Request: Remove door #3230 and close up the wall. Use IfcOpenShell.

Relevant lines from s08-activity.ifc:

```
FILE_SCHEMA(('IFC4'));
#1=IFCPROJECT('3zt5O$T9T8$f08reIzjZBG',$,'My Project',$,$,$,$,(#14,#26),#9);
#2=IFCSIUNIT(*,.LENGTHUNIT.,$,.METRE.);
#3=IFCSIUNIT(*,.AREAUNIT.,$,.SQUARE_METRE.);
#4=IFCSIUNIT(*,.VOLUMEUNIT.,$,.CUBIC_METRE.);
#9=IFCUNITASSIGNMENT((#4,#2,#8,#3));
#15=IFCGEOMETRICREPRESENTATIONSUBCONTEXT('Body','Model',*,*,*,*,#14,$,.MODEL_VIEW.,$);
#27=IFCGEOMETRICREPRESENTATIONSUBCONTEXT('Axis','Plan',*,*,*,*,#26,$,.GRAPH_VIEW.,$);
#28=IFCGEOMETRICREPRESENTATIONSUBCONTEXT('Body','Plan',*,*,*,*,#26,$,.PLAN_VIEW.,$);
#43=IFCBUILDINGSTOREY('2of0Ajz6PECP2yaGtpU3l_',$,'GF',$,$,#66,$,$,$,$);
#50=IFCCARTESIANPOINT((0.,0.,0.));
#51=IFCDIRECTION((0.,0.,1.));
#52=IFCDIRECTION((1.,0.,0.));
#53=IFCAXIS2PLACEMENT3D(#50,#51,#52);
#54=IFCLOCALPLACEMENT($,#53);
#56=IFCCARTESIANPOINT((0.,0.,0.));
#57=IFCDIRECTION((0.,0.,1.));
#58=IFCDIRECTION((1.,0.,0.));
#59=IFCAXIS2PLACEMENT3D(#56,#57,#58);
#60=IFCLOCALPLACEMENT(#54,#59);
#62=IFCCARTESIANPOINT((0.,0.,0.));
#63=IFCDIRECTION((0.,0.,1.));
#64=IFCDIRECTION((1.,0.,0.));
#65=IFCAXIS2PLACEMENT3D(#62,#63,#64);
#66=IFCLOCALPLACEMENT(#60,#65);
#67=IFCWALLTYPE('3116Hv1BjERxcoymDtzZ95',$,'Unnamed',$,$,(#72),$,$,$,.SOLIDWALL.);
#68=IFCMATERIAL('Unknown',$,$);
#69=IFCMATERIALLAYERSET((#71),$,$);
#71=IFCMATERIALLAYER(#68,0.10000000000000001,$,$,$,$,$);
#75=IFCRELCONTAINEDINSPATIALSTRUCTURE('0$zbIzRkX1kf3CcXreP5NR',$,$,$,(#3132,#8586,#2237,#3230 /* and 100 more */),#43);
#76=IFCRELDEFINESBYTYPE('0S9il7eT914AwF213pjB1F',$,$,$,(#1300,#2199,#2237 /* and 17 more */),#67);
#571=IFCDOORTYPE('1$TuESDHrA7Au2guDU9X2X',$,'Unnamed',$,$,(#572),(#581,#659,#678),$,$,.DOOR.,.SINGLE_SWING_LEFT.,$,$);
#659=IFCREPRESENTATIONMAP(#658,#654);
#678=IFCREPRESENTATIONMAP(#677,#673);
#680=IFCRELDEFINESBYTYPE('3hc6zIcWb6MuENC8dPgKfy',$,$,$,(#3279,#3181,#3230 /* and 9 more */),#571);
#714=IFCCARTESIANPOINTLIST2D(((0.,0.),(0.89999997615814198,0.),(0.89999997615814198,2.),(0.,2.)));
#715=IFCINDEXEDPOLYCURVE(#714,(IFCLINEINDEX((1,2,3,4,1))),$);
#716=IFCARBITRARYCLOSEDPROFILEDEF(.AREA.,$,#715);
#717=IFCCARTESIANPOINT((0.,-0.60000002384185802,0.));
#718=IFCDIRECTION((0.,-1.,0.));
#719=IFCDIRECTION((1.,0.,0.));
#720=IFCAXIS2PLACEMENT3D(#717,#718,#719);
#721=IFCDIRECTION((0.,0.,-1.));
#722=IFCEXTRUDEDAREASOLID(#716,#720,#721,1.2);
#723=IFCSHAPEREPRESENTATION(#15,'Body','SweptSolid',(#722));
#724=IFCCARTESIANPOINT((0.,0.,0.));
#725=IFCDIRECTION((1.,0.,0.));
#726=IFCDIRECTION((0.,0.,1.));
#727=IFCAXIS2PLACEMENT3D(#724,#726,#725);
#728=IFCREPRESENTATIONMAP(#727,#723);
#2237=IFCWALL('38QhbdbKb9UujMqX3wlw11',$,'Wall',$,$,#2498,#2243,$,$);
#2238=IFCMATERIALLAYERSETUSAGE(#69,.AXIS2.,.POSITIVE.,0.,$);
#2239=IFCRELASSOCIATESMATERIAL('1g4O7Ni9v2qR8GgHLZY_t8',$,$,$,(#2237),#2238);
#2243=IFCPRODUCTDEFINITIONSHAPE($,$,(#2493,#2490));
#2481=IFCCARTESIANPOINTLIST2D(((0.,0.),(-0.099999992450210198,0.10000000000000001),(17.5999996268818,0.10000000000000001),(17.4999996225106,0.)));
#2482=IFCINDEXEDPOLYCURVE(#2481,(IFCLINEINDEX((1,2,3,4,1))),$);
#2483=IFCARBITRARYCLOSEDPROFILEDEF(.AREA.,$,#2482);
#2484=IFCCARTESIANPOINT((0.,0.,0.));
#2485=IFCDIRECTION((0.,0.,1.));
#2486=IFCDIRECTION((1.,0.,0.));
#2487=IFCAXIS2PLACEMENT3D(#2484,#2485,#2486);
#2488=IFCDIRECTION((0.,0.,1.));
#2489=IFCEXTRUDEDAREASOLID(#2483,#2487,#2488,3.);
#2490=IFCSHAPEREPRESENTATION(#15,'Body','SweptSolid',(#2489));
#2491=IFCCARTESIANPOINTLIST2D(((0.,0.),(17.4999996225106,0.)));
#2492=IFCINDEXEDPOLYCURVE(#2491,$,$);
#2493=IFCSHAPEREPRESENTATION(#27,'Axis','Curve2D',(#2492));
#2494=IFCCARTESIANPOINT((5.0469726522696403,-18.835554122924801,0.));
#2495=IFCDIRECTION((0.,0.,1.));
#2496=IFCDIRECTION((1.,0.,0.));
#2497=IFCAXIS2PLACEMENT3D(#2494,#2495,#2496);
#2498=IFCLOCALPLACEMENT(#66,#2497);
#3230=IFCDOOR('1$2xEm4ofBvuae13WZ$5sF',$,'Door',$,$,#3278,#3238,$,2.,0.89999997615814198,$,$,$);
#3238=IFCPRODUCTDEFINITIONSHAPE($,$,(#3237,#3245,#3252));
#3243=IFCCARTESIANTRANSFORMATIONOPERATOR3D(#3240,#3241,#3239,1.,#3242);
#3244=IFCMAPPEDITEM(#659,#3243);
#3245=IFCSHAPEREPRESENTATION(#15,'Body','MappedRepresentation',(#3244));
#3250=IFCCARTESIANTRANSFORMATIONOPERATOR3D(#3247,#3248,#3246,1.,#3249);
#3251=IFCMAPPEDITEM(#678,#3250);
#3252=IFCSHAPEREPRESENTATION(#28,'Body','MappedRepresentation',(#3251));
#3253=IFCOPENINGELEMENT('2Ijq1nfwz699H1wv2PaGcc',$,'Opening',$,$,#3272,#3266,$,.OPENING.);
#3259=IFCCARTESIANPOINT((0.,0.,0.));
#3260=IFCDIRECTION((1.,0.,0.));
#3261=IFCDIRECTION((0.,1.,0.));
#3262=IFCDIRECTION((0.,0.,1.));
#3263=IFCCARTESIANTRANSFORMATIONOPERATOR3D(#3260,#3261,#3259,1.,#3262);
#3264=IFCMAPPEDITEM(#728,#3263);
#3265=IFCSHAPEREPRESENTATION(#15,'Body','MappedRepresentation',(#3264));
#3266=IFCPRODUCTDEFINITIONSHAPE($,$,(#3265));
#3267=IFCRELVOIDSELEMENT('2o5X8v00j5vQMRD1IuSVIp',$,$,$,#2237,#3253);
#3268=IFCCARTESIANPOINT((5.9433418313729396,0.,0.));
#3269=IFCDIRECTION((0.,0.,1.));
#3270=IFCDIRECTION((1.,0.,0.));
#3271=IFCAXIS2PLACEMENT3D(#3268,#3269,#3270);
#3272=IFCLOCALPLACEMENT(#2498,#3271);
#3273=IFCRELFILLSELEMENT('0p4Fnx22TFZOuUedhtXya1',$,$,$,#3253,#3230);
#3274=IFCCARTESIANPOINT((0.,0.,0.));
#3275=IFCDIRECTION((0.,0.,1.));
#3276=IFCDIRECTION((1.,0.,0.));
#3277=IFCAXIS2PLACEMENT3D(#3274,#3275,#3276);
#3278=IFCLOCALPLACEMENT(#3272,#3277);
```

```python
import ifcopenshell
import ifcopenshell.api.feature
import ifcopenshell.api.root
import ifcopenshell.geom
import ifcopenshell.util.shape

model = ifcopenshell.open("s08-activity.ifc")
settings = ifcopenshell.geom.settings()


def volume(element):
    """Net volume in cubic metres, openings subtracted."""
    shape = ifcopenshell.geom.create_shape(settings, element)
    return ifcopenshell.util.shape.get_volume(shape.geometry)


door = model.by_id(3230)
opening = door.FillsVoids[0].RelatingOpeningElement
wall = opening.VoidsElements[0].RelatingBuildingElement
before = volume(wall)

ifcopenshell.api.root.remove_product(model, product=door)
ifcopenshell.api.feature.remove_feature(model, feature=opening)

after = volume(wall)

print(f"wall volume {before:.3f} -> {after:.3f} m3")

model.write("s08-activity_rev.ifc")
```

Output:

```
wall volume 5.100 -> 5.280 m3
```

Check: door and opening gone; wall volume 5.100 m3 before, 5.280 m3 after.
